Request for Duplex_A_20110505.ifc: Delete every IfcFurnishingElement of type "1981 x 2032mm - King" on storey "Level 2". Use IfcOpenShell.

First a look at what the model holds.

```python
import ifcopenshell
import ifcopenshell.util.element

model = ifcopenshell.open("Duplex_A_20110505.ifc")
print(model.schema)
storey = next(s for s in model.by_type("IfcBuildingStorey") if s.Name == "Level 2")
furniture = [e for e in ifcopenshell.util.element.get_decomposition(storey) if e.is_a("IfcFurnishingElement")]
seen = {}
for e in furniture:
    element_type = ifcopenshell.util.element.get_type(e)
    name = element_type.Name if element_type not in (None, e) else None
    seen[name] = seen.get(name, 0) + 1
for name, count in sorted(seen.items(), key=str):
    print(count, "x", name)
```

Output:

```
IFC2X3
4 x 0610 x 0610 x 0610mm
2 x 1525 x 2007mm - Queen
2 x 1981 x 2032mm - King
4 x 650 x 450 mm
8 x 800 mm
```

```python
import ifcopenshell
import ifcopenshell.api.root
import ifcopenshell.util.element

model = ifcopenshell.open("Duplex_A_20110505.ifc")

storey = next(s for s in model.by_type("IfcBuildingStorey") if s.Name == "Level 2")
furniture = [e for e in ifcopenshell.util.element.get_decomposition(storey) if e.is_a("IfcFurnishingElement")]
targets = [e for e in furniture if (t := ifcopenshell.util.element.get_type(e)) not in (None, e) and t.Name == "1981 x 2032mm - King"]

for e in targets:
    ifcopenshell.api.root.remove_product(model, product=e)
print(len(targets), "removed")

model.write("Duplex_A_20110505_v2.ifc")
```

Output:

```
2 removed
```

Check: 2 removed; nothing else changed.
